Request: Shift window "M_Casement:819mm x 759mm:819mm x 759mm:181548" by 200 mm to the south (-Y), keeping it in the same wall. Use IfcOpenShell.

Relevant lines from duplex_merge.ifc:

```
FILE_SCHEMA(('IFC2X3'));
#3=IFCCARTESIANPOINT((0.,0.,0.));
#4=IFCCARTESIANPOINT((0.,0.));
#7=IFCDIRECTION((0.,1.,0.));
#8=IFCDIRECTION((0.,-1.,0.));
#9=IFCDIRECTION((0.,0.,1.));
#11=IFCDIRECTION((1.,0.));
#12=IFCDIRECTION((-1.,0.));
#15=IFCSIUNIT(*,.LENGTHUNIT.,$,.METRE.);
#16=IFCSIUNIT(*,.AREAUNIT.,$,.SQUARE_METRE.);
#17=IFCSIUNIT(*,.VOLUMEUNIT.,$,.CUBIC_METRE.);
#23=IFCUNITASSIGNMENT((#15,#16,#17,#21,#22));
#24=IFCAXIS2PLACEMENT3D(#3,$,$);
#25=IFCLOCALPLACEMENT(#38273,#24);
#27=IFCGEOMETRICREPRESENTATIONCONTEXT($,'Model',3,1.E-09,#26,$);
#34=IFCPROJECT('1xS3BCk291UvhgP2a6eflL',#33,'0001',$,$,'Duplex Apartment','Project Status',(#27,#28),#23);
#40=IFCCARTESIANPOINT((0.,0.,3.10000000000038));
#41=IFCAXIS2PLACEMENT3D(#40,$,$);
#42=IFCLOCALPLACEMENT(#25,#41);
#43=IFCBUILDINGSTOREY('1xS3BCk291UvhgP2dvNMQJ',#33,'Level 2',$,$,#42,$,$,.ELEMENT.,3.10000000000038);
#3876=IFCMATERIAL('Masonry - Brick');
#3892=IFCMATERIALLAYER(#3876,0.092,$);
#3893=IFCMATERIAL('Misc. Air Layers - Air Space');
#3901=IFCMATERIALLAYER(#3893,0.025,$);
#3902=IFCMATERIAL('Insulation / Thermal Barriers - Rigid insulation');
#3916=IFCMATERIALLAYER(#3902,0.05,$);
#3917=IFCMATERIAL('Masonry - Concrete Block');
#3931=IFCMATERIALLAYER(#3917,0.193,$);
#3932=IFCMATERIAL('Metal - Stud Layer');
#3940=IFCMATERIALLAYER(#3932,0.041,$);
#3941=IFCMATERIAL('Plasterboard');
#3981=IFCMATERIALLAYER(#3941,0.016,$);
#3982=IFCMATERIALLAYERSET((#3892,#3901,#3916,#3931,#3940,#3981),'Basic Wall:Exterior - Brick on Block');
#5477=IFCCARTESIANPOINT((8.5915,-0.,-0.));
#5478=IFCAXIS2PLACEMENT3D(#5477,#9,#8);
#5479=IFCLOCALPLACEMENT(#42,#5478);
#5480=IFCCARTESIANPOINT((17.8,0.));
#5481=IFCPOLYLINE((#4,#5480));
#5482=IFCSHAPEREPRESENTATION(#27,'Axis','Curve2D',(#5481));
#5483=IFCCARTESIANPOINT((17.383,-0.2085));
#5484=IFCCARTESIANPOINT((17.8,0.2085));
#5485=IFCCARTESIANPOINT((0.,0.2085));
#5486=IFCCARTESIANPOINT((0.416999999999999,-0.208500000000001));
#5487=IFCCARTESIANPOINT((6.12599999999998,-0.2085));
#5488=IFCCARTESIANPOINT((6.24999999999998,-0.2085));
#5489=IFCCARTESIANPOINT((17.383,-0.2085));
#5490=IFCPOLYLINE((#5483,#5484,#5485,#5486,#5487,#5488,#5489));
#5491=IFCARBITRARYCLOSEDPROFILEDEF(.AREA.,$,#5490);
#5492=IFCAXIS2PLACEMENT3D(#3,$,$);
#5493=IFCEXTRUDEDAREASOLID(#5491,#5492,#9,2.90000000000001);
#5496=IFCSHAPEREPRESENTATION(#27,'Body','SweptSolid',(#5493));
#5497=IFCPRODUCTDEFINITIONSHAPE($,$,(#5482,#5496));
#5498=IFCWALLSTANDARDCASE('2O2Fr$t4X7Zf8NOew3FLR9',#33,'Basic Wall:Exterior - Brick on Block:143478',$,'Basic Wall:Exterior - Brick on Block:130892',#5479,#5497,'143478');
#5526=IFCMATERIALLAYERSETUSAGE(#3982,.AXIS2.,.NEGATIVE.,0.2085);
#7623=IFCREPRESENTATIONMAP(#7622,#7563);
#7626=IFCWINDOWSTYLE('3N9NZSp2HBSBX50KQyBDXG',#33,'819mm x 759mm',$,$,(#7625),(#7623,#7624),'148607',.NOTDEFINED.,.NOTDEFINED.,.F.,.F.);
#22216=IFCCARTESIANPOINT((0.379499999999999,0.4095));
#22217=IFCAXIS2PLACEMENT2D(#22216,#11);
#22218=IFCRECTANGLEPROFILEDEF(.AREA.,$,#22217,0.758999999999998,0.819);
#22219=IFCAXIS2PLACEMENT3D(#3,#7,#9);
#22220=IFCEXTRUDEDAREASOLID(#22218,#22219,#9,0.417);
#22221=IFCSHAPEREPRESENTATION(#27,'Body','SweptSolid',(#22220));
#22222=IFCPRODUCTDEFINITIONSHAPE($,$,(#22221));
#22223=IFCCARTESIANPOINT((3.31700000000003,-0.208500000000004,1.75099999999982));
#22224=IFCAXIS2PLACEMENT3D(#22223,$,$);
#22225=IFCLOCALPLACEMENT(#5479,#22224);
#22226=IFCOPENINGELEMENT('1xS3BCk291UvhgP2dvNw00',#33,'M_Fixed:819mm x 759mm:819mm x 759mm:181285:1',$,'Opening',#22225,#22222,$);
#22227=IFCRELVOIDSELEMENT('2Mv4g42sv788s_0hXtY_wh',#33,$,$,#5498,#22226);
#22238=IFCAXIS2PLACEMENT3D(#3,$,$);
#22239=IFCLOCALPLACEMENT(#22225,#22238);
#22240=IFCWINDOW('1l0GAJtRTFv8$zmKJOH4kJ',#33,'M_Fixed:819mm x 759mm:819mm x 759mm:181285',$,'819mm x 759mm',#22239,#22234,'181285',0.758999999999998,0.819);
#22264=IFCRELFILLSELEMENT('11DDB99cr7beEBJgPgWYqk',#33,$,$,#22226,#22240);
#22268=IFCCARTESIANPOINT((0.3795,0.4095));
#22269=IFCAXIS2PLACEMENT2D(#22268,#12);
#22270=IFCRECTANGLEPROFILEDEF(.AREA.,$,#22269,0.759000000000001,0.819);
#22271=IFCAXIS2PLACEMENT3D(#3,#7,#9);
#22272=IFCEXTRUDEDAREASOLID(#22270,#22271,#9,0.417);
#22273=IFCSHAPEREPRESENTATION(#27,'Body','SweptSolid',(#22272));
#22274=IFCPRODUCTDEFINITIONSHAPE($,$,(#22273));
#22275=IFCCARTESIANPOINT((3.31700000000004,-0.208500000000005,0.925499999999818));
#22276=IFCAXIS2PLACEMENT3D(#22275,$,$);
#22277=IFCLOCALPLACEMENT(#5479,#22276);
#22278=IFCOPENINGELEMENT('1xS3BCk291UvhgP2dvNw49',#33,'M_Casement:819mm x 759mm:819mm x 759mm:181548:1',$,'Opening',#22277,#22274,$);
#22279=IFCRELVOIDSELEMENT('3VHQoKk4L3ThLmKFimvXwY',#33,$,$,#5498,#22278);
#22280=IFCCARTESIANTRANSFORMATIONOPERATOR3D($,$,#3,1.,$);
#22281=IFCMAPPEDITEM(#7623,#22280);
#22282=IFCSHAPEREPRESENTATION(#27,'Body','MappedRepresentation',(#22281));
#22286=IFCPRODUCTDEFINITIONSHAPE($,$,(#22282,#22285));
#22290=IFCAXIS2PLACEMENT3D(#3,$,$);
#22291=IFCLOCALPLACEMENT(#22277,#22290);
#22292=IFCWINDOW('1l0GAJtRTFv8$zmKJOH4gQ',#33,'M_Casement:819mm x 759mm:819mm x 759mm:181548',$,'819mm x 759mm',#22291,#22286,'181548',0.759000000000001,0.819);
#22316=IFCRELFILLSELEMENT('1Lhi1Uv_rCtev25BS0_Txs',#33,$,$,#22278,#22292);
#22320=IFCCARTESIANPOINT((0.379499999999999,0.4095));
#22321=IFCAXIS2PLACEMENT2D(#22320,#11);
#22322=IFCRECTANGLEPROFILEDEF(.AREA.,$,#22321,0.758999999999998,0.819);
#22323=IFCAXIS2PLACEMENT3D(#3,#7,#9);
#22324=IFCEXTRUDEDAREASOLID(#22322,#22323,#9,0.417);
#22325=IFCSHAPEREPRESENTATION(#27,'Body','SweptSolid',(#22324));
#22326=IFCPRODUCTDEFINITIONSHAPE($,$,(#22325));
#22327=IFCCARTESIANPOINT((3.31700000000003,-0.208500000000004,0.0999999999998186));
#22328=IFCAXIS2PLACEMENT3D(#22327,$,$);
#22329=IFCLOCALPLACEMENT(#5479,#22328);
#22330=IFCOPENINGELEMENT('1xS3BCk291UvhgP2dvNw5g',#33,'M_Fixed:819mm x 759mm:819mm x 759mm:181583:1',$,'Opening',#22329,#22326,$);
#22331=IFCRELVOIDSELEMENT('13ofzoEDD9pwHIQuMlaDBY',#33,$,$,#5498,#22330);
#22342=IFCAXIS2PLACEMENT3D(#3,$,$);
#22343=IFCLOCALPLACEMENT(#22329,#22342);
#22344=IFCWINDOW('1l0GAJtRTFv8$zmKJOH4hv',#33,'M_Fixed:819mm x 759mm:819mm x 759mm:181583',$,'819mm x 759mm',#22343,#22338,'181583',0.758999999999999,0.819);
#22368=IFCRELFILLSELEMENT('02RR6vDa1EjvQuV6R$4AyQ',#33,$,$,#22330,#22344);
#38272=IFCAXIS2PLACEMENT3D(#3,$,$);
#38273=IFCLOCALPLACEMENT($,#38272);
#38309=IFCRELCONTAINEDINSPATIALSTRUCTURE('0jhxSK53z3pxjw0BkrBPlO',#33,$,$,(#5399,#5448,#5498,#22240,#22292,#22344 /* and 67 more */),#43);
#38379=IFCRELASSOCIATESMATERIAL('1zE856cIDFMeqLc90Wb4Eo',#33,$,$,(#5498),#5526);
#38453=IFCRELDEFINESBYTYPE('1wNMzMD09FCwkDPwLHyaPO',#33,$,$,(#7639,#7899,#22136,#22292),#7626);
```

```python
import ifcopenshell
import ifcopenshell.api.geometry
import ifcopenshell.util.placement

model = ifcopenshell.open("duplex_merge.ifc")

window = model.by_guid("1l0GAJtRTFv8$zmKJOH4gQ")
opening = window.FillsVoids[0].RelatingOpeningElement
wall = opening.VoidsElements[0].RelatingBuildingElement

wall_matrix = ifcopenshell.util.placement.get_local_placement(wall.ObjectPlacement)
shift = wall_matrix[:3, 0] * 0.2
before = ifcopenshell.util.placement.get_local_placement(window.ObjectPlacement)[:3, 3].copy()

# The window is placed relative to its opening, so it follows when the opening moves.
matrix = ifcopenshell.util.placement.get_local_placement(opening.ObjectPlacement)
matrix[:3, 3] += shift
ifcopenshell.api.geometry.edit_object_placement(
    model, product=opening, matrix=matrix, is_si=False, should_transform_children=True
)

after = ifcopenshell.util.placement.get_local_placement(window.ObjectPlacement)[:3, 3]
print("window moved by", (after - before).round(3) + 0.0)

model.write("duplex_merge_updated.ifc")
```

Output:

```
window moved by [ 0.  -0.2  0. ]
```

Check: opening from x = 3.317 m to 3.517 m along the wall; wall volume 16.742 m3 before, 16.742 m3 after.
